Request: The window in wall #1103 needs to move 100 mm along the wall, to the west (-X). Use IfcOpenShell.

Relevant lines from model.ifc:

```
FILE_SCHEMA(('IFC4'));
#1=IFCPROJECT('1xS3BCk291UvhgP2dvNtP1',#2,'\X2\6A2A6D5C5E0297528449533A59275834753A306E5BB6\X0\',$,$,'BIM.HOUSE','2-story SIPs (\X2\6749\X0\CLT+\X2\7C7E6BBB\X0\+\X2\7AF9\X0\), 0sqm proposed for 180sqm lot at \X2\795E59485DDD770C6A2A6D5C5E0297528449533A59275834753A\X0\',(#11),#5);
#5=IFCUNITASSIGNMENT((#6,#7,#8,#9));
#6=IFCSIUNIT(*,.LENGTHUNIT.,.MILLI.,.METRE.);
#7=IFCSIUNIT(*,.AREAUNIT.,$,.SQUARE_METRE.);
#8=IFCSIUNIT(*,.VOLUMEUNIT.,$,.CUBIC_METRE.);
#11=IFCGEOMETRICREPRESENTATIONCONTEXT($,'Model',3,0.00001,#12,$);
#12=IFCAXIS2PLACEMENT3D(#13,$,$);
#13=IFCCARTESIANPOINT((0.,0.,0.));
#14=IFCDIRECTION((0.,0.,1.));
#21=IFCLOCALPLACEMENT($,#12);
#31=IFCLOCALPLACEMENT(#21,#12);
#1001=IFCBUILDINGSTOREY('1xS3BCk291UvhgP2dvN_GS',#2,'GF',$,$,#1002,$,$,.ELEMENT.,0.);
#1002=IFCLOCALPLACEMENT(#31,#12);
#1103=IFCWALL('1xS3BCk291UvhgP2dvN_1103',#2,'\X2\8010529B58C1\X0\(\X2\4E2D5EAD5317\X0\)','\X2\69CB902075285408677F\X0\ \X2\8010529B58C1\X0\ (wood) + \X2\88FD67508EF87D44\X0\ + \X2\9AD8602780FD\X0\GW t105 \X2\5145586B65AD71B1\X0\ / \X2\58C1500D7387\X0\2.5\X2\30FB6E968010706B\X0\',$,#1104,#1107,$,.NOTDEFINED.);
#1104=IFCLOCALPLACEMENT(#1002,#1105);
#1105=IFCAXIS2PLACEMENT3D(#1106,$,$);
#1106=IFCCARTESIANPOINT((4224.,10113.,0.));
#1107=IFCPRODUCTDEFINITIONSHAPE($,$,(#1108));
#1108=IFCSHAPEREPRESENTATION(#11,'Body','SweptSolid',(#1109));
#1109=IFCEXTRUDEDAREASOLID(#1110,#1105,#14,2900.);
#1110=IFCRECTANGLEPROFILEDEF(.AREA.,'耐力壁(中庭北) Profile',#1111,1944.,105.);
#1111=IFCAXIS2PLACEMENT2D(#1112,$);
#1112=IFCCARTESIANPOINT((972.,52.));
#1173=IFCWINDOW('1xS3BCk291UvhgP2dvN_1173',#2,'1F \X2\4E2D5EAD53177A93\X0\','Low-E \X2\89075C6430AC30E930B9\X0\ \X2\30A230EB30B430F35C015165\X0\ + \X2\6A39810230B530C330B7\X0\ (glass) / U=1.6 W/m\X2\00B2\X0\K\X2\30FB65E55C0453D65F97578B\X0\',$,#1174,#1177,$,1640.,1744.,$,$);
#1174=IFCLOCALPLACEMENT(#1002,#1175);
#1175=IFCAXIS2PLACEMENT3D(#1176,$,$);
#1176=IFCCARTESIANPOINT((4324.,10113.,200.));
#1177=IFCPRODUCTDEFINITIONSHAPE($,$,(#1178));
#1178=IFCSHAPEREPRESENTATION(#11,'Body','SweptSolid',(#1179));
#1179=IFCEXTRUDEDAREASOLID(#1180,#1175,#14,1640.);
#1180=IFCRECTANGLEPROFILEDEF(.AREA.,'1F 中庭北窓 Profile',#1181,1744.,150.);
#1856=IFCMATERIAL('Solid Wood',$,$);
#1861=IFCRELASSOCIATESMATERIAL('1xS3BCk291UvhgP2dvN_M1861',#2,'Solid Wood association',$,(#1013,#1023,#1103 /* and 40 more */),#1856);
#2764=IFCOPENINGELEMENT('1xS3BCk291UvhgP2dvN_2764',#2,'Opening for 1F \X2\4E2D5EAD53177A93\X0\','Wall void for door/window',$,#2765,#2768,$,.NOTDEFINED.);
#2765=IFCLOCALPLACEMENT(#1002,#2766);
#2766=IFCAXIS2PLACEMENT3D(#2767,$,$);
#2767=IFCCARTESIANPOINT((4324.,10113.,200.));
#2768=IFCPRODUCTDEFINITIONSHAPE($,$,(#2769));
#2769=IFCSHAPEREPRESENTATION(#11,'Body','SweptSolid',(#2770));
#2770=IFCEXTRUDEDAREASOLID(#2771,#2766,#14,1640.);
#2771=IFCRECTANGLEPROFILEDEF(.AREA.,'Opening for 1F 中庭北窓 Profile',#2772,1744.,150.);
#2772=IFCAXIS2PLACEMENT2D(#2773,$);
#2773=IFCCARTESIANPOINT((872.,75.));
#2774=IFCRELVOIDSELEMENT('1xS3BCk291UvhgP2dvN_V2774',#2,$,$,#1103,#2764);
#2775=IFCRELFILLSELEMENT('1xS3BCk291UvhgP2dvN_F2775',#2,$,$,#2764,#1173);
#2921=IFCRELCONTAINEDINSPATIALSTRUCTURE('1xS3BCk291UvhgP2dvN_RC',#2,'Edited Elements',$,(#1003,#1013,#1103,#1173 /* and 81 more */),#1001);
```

```python
import ifcopenshell
import ifcopenshell.api.geometry
import ifcopenshell.util.placement

model = ifcopenshell.open("model.ifc")

window = model.by_id(1173)
opening = window.FillsVoids[0].RelatingOpeningElement
wall = opening.VoidsElements[0].RelatingBuildingElement

wall_matrix = ifcopenshell.util.placement.get_local_placement(wall.ObjectPlacement)
shift = wall_matrix[:3, 0] * -100.0
before = ifcopenshell.util.placement.get_local_placement(window.ObjectPlacement)[:3, 3].copy()

# The window is not placed relative to its opening, so move both.
for product in (opening, window):
    matrix = ifcopenshell.util.placement.get_local_placement(product.ObjectPlacement)
    matrix[:3, 3] += shift
    ifcopenshell.api.geometry.edit_object_placement(model, product=product, matrix=matrix, is_si=False)

after = ifcopenshell.util.placement.get_local_placement(window.ObjectPlacement)[:3, 3]
print("window moved by", (after - before).round(3) + 0.0)

model.write("model_updated.ifc")
```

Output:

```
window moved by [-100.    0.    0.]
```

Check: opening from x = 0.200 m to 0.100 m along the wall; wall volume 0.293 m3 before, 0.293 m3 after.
